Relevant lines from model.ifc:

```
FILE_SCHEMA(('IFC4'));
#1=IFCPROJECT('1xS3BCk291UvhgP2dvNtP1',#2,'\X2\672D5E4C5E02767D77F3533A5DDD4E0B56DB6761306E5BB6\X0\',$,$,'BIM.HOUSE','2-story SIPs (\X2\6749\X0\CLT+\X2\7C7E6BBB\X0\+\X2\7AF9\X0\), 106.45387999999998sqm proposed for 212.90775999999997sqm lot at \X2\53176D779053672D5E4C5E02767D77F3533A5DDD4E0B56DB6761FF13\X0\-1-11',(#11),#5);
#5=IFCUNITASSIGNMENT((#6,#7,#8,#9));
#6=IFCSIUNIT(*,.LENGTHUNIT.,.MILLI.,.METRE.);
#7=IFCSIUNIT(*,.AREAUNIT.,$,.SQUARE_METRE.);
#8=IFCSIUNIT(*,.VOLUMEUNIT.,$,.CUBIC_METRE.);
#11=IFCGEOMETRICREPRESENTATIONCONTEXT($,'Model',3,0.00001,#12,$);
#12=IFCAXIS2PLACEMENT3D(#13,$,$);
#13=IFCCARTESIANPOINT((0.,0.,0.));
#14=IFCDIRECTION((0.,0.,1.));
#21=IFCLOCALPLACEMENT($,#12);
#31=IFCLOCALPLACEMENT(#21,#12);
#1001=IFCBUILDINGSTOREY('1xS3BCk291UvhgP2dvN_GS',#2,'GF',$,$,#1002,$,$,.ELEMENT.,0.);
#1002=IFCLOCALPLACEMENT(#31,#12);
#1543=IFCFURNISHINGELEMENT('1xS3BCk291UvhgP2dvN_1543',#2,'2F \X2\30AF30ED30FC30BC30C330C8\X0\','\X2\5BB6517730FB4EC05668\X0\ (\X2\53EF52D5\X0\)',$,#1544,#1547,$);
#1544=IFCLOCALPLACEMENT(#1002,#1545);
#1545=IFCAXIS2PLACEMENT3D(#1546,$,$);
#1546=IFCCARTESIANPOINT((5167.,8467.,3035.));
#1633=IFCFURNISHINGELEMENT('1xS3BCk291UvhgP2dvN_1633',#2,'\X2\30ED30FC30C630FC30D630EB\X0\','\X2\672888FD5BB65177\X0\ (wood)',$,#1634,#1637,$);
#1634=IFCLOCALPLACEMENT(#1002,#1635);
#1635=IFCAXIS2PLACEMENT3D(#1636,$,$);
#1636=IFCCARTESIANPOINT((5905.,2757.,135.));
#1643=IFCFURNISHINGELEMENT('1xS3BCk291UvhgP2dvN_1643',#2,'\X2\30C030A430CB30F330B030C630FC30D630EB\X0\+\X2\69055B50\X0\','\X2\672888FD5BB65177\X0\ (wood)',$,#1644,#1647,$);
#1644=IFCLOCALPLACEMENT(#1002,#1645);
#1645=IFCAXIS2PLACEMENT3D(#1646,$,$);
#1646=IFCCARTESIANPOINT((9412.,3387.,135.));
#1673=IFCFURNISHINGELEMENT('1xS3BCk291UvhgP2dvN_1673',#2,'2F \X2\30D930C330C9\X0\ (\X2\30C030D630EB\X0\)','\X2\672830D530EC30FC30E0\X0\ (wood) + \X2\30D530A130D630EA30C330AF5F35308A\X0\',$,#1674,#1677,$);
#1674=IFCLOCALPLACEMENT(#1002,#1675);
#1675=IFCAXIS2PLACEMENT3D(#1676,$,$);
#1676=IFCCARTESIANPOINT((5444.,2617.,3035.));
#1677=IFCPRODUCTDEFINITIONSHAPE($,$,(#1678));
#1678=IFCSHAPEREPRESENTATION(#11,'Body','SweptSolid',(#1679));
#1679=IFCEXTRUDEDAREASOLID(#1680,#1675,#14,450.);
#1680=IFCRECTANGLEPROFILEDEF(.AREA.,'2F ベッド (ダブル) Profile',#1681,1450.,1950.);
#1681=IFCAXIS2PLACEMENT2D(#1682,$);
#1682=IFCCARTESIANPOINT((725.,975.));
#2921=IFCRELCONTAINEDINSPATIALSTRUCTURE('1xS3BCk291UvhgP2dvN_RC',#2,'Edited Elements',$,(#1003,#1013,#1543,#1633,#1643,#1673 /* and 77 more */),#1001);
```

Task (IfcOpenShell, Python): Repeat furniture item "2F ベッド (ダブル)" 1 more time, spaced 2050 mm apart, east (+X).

```python
import numpy as np
import ifcopenshell
import ifcopenshell.api.geometry
import ifcopenshell.api.root
import ifcopenshell.util.element
import ifcopenshell.util.placement
import ifcopenshell.util.unit

model = ifcopenshell.open("model.ifc")
unit_scale = ifcopenshell.util.unit.calculate_unit_scale(model)


def reuse_history(source, copy):
    """copy_class also copies each property set's owner history, people and application; keep the originals."""
    for rel in copy.IsDefinedBy:
        if rel.is_a("IfcRelDefinesByProperties") and (history := rel.RelatingPropertyDefinition.OwnerHistory):
            rel.RelatingPropertyDefinition.OwnerHistory = source.OwnerHistory
            ifcopenshell.util.element.remove_deep2(model, history)


source = model.by_guid("1xS3BCk291UvhgP2dvN_1673")
base = ifcopenshell.util.placement.get_local_placement(source.ObjectPlacement)
step = np.array([1.0, 0.0, 0.0]) * 2.05 / unit_scale

for i in range(1, 2):
    copy = ifcopenshell.api.root.copy_class(model, product=source)
    copy.Representation = ifcopenshell.util.element.copy_deep(
        model, source.Representation, exclude=["IfcGeometricRepresentationContext", "IfcRepresentationMap"]
    )
    reuse_history(source, copy)
    matrix = base.copy()
    matrix[:3, 3] += i * step
    print("added at", matrix[:3, 3].round(3) + 0.0)
    ifcopenshell.api.geometry.edit_object_placement(model, product=copy, matrix=matrix, is_si=False)

model.write("model_rev.ifc")
```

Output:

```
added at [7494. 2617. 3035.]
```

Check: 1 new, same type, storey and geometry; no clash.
